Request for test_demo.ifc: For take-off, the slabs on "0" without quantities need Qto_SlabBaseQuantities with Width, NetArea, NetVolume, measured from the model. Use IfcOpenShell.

First a look at what the model holds.

```python
import ifcopenshell
import ifcopenshell.util.element
import ifcopenshell.util.unit

model = ifcopenshell.open("test_demo.ifc")
print(model.schema)
for unit_type in ("LENGTHUNIT", "AREAUNIT", "VOLUMEUNIT"):
    print(unit_type, ifcopenshell.util.unit.calculate_unit_scale(model, unit_type))
storey = next(s for s in model.by_type("IfcBuildingStorey") if s.Name == "0")
slabs = [e for e in ifcopenshell.util.element.get_decomposition(storey) if e.is_a("IfcSlab")]
for e in sorted(slabs, key=lambda e: e.id()):
    print(e.id(), e.is_a(), e.Name, list(ifcopenshell.util.element.get_psets(e, qtos_only=True)), sep=" | ")
```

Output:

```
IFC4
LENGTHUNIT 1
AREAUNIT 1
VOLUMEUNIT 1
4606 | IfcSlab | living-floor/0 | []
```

```python
import ifcopenshell
import ifcopenshell.api.pset
import ifcopenshell.geom
import ifcopenshell.util.element
import ifcopenshell.util.shape
import ifcopenshell.util.unit

model = ifcopenshell.open("test_demo.ifc")
unit_scale = ifcopenshell.util.unit.calculate_unit_scale(model)
area_scale = ifcopenshell.util.unit.calculate_unit_scale(model, "AREAUNIT")
volume_scale = ifcopenshell.util.unit.calculate_unit_scale(model, "VOLUMEUNIT")
settings = ifcopenshell.geom.settings()

storey = next(s for s in model.by_type("IfcBuildingStorey") if s.Name == "0")
slabs = [e for e in ifcopenshell.util.element.get_decomposition(storey) if e.is_a("IfcSlab")]

for e in sorted(slabs, key=lambda e: e.id()):
    if ifcopenshell.util.element.get_psets(e, qtos_only=True, should_inherit=False):
        continue
    # Geometry comes back in metres, in the element's own axes.
    shape = ifcopenshell.geom.create_shape(settings, e)
    values = {
        "Width": ifcopenshell.util.shape.get_z(shape.geometry) / unit_scale,
        "NetArea": ifcopenshell.util.shape.get_footprint_area(shape.geometry) / area_scale,
        "NetVolume": ifcopenshell.util.shape.get_volume(shape.geometry) / volume_scale,
    }
    qto = ifcopenshell.api.pset.add_qto(model, product=e, name="Qto_SlabBaseQuantities")
    ifcopenshell.api.pset.edit_qto(model, qto=qto, properties=values)
    print(e.id(), {k: round(v, 3) for k, v in values.items()})

model.write("test_demo-out.ifc")
```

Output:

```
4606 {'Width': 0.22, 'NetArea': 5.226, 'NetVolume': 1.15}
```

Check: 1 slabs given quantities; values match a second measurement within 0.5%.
